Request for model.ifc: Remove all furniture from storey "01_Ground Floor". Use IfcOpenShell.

First a look at what the model holds.

```python
import ifcopenshell
import ifcopenshell.util.element

model = ifcopenshell.open("model.ifc")
print(model.schema)
storey = next(s for s in model.by_type("IfcBuildingStorey") if s.Name == "01_Ground Floor")
furniture = [e for e in ifcopenshell.util.element.get_decomposition(storey) if e.is_a("IfcFurnishingElement")]
seen = {}
for e in furniture:
    element_type = ifcopenshell.util.element.get_type(e)
    name = element_type.Name if element_type not in (None, e) else None
    seen[name] = seen.get(name, 0) + 1
for name, count in sorted(seen.items(), key=str):
    print(count, "x", name)
```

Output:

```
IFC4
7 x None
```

```python
import ifcopenshell
import ifcopenshell.api.root
import ifcopenshell.util.element

model = ifcopenshell.open("model.ifc")

storey = next(s for s in model.by_type("IfcBuildingStorey") if s.Name == "01_Ground Floor")
furniture = [e for e in ifcopenshell.util.element.get_decomposition(storey) if e.is_a("IfcFurnishingElement")]

for e in furniture:
    ifcopenshell.api.root.remove_product(model, product=e)
print(len(furniture), "removed")

model.write("model_rev.ifc")
```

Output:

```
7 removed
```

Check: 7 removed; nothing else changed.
